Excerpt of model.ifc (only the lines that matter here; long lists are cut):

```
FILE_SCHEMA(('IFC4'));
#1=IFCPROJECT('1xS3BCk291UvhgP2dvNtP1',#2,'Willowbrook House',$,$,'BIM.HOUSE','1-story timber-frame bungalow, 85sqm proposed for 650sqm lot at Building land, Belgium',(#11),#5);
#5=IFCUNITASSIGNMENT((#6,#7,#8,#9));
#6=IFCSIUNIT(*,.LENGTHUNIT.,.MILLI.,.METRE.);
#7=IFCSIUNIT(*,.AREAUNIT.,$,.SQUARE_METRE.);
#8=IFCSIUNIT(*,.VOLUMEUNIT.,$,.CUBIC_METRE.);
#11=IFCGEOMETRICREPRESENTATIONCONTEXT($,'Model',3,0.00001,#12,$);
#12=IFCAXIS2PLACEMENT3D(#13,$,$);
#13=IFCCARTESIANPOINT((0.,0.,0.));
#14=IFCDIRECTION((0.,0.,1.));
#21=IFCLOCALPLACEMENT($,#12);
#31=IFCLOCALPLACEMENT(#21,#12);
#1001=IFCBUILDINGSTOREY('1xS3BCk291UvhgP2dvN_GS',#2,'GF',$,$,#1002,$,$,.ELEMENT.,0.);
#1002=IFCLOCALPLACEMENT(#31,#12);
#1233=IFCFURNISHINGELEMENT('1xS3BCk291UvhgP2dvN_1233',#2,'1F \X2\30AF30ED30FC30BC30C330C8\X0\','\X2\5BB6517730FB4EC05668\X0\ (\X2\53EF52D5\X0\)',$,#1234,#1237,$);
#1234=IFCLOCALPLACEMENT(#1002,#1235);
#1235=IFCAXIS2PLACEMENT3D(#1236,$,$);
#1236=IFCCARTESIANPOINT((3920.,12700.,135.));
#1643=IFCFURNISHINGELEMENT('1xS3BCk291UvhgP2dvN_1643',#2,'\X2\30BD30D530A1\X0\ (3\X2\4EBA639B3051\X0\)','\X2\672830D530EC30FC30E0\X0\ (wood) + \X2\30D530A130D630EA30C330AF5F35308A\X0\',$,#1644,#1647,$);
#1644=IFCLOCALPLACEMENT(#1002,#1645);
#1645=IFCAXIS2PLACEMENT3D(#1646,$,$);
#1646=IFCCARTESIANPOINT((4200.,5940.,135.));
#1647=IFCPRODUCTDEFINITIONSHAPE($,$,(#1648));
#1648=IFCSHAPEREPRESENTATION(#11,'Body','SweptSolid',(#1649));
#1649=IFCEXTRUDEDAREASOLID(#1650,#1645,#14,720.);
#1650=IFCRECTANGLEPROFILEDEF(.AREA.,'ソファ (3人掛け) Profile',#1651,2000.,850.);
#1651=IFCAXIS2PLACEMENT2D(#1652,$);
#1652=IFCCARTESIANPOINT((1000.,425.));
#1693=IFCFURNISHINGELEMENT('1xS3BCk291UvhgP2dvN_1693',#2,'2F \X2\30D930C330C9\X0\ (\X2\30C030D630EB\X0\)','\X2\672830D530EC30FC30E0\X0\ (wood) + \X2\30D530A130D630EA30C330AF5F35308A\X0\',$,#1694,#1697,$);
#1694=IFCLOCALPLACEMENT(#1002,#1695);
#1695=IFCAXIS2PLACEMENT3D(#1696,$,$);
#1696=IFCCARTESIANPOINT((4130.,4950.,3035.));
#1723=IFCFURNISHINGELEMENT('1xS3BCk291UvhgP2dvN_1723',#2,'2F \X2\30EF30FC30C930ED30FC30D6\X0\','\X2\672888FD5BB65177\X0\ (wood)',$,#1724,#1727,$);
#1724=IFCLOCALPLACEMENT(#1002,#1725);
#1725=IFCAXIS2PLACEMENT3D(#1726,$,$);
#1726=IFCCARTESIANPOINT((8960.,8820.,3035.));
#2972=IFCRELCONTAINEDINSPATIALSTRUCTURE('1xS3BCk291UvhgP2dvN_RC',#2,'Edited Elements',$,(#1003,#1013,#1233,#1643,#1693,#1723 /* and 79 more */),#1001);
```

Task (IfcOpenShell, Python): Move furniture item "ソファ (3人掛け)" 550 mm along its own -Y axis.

```python
import ifcopenshell
import ifcopenshell.api.geometry
import ifcopenshell.util.placement
import ifcopenshell.util.unit

model = ifcopenshell.open("model.ifc")
unit_scale = ifcopenshell.util.unit.calculate_unit_scale(model)

item = model.by_guid("1xS3BCk291UvhgP2dvN_1643")
matrix = ifcopenshell.util.placement.get_local_placement(item.ObjectPlacement)
matrix[:3, 3] -= matrix[:3, 1] * 0.55 / unit_scale
ifcopenshell.api.geometry.edit_object_placement(model, product=item, matrix=matrix, is_si=False)

print(ifcopenshell.util.placement.get_local_placement(item.ObjectPlacement).round(3) + 0.0)

model.write("model-out.ifc")
```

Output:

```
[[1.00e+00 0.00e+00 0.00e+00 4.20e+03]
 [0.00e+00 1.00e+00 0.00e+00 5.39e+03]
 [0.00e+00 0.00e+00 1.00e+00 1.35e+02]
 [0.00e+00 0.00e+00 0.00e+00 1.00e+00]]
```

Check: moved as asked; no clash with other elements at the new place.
